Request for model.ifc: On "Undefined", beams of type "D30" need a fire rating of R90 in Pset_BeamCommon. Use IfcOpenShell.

First a look at what the model holds.

```python
import ifcopenshell
import ifcopenshell.util.element

model = ifcopenshell.open("model.ifc")
print(model.schema)
storey = next(s for s in model.by_type("IfcBuildingStorey") if s.Name == "Undefined")
beams = [e for e in ifcopenshell.util.element.get_decomposition(storey) if e.is_a("IfcBeam")]
seen = {}
for e in beams:
    element_type = ifcopenshell.util.element.get_type(e)
    key = (element_type.Name if element_type != e and element_type else None, ifcopenshell.util.element.get_pset(e, "Pset_BeamCommon", "FireRating"))
    seen[key] = seen.get(key, 0) + 1
for (name, value), count in sorted(seen.items(), key=str):
    print(count, "x", name, "|", value)
```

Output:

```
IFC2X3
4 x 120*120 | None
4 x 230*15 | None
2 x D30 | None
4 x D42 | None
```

```python
import ifcopenshell
import ifcopenshell.api.pset
import ifcopenshell.util.element

model = ifcopenshell.open("model.ifc")

storey = next(s for s in model.by_type("IfcBuildingStorey") if s.Name == "Undefined")
beams = [e for e in ifcopenshell.util.element.get_decomposition(storey) if e.is_a("IfcBeam")]

count = 0
for e in beams:
    element_type = ifcopenshell.util.element.get_type(e)
    if element_type in (None, e) or element_type.Name != "D30":
        continue
    # add_pset returns the element's existing set when there is one.
    pset = ifcopenshell.api.pset.add_pset(model, product=e, name="Pset_BeamCommon")
    ifcopenshell.api.pset.edit_pset(model, pset=pset, properties={"FireRating": "R90"})
    count += 1

print(count, "beams updated")

model.write("model_rev.ifc")
```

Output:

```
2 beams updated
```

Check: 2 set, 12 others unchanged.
